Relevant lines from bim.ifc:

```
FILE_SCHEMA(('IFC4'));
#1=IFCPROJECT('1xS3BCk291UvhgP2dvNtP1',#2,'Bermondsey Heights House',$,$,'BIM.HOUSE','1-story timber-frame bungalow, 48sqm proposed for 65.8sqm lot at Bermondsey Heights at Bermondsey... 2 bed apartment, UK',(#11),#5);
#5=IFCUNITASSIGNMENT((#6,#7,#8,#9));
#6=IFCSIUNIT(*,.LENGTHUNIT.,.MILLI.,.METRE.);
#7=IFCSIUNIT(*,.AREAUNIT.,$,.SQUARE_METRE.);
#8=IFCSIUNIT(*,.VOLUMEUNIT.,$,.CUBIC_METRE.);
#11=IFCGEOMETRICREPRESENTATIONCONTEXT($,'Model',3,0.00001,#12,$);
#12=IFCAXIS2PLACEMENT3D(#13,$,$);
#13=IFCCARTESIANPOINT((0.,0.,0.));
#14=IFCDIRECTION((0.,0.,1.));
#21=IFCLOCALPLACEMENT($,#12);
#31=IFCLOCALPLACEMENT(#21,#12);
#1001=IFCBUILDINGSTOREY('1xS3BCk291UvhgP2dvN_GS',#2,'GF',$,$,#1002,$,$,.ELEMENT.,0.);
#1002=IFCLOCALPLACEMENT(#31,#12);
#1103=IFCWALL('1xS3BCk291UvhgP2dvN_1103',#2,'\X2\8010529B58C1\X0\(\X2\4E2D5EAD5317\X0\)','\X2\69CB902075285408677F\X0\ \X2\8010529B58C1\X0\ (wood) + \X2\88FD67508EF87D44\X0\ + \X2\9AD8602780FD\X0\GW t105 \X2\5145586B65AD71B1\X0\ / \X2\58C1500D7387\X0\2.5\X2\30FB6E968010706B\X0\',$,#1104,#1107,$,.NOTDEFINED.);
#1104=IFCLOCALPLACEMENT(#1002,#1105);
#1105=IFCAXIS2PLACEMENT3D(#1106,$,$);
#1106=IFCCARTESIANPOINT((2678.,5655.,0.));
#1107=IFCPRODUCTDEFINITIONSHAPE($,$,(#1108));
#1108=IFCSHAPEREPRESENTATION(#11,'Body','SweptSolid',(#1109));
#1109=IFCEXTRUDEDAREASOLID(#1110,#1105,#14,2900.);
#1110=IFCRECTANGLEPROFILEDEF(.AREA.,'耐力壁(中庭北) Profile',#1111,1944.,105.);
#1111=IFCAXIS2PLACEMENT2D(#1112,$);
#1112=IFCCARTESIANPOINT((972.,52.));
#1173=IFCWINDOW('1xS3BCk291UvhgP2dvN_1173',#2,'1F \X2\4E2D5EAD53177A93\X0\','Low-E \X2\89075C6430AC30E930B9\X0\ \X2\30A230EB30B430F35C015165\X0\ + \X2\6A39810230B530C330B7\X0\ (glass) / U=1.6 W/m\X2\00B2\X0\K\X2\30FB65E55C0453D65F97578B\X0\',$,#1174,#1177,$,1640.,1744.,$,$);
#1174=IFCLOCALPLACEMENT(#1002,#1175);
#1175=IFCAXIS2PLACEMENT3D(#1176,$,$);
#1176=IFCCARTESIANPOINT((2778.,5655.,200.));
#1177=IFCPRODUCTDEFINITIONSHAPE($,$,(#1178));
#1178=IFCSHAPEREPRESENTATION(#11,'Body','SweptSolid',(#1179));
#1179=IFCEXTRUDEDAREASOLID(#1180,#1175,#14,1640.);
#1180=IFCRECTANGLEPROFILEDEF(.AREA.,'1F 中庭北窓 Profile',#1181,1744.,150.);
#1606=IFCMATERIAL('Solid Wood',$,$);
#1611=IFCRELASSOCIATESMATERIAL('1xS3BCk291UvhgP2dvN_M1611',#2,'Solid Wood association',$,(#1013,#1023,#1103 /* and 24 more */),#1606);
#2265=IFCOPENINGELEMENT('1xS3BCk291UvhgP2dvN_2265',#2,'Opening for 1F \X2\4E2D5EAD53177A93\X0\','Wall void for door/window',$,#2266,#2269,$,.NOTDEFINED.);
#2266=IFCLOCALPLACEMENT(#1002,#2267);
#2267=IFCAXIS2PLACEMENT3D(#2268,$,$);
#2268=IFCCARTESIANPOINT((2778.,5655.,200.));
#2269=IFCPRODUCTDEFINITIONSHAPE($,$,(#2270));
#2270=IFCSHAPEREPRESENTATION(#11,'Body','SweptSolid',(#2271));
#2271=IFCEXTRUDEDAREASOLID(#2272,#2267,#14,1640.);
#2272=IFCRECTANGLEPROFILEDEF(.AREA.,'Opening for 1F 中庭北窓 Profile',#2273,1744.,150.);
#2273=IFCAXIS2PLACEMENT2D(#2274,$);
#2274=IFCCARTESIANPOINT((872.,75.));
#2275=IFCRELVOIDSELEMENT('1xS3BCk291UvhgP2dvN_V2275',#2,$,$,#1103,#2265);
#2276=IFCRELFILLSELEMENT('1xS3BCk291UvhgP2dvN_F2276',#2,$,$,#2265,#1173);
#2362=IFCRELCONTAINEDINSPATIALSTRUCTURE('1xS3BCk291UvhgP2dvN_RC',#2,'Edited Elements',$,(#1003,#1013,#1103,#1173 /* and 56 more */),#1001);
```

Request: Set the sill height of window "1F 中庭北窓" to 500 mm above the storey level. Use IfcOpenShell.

```python
import numpy as np
import ifcopenshell
import ifcopenshell.api.geometry
import ifcopenshell.geom
import ifcopenshell.util.element
import ifcopenshell.util.placement
import ifcopenshell.util.shape
import ifcopenshell.util.unit

model = ifcopenshell.open("bim.ifc")
unit_scale = ifcopenshell.util.unit.calculate_unit_scale(model)

window = model.by_guid("1xS3BCk291UvhgP2dvN_1173")
opening = window.FillsVoids[0].RelatingOpeningElement
storey = ifcopenshell.util.element.get_container(window, ifc_class="IfcBuildingStorey")
level = ifcopenshell.util.placement.get_local_placement(storey.ObjectPlacement)[2, 3]

# The opening's origin need not be at the sill, so measure its lowest point.
shape = ifcopenshell.geom.create_shape(ifcopenshell.geom.settings(), opening)
bottom = ifcopenshell.util.shape.get_shape_bottom_elevation(shape, shape.geometry) / unit_scale
dz = level + 0.5 / unit_scale - bottom

shift = np.array([0.0, 0.0, dz])
# The window is not placed relative to its opening, so move both.
for product in (opening, window):
    matrix = ifcopenshell.util.placement.get_local_placement(product.ObjectPlacement)
    matrix[:3, 3] += shift
    ifcopenshell.api.geometry.edit_object_placement(model, product=product, matrix=matrix, is_si=False)

print(f"moved by {dz * unit_scale:+.3f} m")

model.write("bim_updated.ifc")
```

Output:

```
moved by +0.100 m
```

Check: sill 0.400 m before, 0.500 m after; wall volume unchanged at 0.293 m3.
